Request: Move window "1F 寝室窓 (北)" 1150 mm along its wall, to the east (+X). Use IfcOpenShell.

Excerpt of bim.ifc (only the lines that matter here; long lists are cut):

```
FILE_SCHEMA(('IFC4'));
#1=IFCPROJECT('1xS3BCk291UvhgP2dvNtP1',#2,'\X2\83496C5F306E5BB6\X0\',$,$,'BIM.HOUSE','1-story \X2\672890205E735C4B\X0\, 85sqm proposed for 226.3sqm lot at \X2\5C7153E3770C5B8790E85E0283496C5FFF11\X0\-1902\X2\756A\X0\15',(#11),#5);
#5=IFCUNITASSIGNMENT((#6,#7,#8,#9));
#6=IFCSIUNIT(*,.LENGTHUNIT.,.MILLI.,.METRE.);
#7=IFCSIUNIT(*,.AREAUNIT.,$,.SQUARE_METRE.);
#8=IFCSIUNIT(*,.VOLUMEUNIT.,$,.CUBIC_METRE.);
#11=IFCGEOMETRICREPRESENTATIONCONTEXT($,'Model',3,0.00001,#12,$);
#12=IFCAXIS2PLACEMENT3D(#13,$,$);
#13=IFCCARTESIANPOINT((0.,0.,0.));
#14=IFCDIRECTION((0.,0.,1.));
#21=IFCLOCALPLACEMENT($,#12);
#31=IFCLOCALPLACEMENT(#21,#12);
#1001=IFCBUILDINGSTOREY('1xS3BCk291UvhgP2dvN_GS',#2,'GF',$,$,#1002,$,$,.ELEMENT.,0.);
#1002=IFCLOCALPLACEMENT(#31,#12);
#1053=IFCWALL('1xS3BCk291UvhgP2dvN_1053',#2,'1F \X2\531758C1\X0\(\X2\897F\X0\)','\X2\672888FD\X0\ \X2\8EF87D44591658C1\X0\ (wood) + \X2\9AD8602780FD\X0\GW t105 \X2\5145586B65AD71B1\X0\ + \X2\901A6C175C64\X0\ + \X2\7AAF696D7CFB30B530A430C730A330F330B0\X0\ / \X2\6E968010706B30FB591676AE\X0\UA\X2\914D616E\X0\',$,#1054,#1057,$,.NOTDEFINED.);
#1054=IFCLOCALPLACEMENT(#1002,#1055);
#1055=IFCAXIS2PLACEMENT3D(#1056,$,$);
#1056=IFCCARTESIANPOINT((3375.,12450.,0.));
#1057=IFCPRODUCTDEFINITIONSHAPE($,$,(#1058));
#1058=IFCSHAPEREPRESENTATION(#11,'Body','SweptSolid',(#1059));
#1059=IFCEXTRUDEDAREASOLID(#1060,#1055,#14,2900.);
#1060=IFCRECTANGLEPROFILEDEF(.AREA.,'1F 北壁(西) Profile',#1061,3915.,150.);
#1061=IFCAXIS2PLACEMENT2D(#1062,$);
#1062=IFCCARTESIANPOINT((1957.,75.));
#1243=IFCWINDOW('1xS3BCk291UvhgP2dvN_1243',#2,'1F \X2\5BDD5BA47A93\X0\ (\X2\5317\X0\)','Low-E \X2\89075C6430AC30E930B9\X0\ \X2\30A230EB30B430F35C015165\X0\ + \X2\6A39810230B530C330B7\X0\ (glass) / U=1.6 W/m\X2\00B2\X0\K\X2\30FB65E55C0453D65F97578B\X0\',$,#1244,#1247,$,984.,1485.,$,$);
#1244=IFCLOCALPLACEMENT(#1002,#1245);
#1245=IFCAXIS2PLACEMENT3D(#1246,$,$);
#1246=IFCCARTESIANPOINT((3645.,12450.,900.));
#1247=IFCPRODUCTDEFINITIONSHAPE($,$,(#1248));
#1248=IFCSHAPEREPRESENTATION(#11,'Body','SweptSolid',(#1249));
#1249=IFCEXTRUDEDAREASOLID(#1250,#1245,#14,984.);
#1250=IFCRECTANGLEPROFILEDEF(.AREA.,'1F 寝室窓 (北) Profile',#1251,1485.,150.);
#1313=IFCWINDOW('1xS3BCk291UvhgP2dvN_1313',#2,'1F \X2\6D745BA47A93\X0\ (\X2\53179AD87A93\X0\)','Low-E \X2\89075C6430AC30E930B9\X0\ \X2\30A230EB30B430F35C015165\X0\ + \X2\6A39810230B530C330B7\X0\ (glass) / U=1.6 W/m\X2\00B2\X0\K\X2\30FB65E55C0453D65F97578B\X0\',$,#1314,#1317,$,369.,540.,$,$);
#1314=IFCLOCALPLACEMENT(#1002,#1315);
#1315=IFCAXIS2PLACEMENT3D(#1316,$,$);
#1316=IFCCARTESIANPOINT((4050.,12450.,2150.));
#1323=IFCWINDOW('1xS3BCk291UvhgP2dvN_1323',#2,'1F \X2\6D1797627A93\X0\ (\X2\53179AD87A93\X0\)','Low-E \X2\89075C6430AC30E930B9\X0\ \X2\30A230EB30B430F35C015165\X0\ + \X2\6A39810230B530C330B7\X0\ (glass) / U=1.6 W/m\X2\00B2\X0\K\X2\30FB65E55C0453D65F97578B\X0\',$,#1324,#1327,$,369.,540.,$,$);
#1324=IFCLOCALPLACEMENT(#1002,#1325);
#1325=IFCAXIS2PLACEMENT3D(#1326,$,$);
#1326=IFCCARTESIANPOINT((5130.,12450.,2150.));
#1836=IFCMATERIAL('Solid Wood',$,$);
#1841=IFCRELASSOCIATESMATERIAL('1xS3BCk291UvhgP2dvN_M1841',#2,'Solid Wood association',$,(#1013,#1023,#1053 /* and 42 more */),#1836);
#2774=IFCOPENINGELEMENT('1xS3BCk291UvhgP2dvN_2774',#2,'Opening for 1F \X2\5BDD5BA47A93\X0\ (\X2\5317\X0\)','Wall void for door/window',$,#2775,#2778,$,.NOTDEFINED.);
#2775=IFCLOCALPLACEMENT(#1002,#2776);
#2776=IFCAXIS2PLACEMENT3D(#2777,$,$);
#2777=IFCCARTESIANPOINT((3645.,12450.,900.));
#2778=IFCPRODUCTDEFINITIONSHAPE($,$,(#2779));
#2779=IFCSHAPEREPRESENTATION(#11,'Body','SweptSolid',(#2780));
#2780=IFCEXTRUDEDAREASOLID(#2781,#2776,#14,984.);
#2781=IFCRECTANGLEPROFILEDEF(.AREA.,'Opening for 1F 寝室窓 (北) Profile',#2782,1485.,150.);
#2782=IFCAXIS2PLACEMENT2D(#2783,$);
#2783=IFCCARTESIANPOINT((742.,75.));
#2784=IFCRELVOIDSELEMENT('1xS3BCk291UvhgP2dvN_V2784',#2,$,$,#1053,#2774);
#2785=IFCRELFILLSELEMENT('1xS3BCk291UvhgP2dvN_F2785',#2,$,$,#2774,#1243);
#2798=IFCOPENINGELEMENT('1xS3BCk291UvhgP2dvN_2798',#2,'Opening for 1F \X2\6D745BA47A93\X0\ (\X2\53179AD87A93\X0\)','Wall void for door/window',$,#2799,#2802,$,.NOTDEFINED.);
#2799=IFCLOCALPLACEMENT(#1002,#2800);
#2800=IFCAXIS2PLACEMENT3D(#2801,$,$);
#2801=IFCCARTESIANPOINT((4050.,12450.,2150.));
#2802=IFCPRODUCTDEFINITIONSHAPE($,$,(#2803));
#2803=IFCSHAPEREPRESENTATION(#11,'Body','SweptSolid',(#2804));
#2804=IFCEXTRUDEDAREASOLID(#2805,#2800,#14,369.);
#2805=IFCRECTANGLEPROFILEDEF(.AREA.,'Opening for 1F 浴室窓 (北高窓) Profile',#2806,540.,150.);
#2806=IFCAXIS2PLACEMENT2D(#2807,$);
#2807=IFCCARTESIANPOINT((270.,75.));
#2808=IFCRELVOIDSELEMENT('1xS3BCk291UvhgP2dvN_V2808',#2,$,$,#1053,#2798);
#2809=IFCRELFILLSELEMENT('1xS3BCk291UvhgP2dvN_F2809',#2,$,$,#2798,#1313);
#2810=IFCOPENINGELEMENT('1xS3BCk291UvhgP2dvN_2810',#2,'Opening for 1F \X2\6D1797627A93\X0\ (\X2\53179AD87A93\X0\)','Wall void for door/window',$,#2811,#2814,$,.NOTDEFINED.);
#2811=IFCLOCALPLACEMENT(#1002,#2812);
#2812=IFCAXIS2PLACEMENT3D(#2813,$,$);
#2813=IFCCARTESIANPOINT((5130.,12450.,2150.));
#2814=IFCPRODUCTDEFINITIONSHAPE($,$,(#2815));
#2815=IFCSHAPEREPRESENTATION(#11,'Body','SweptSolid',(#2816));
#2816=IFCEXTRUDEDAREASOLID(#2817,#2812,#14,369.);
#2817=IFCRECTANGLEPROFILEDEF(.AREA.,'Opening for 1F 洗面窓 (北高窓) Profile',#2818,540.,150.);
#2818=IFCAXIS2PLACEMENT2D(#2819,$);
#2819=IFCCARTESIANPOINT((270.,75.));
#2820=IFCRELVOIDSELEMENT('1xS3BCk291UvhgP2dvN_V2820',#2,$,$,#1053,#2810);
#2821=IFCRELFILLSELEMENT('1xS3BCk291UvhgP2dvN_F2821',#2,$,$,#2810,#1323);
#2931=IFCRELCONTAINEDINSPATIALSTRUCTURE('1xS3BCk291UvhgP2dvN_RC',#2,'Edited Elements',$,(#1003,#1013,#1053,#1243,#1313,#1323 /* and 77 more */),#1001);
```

```python
import ifcopenshell
import ifcopenshell.api.geometry
import ifcopenshell.util.placement

model = ifcopenshell.open("bim.ifc")

window = model.by_id(1243)
opening = window.FillsVoids[0].RelatingOpeningElement
wall = opening.VoidsElements[0].RelatingBuildingElement

wall_matrix = ifcopenshell.util.placement.get_local_placement(wall.ObjectPlacement)
shift = wall_matrix[:3, 0] * 1150.0
before = ifcopenshell.util.placement.get_local_placement(window.ObjectPlacement)[:3, 3].copy()

# The window is not placed relative to its opening, so move both.
for product in (opening, window):
    matrix = ifcopenshell.util.placement.get_local_placement(product.ObjectPlacement)
    matrix[:3, 3] += shift
    ifcopenshell.api.geometry.edit_object_placement(model, product=product, matrix=matrix, is_si=False)

after = ifcopenshell.util.placement.get_local_placement(window.ObjectPlacement)[:3, 3]
print("window moved by", (after - before).round(3) + 0.0)

model.write("bim_updated.ifc")
```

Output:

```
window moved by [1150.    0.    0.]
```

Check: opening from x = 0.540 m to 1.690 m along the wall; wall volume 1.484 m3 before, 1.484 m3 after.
